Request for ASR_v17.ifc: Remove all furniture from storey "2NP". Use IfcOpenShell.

First a look at what the model holds.

```python
import ifcopenshell
import ifcopenshell.util.element

model = ifcopenshell.open("ASR_v17.ifc")
print(model.schema)
storey = next(s for s in model.by_type("IfcBuildingStorey") if s.Name == "2NP")
furniture = [e for e in ifcopenshell.util.element.get_decomposition(storey) if e.is_a("IfcFurnishingElement")]
seen = {}
for e in furniture:
    element_type = ifcopenshell.util.element.get_type(e)
    name = element_type.Name if element_type not in (None, e) else None
    seen[name] = seen.get(name, 0) + 1
for name, count in sorted(seen.items(), key=str):
    print(count, "x", name)
```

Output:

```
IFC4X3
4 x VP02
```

```python
import ifcopenshell
import ifcopenshell.api.root
import ifcopenshell.util.element

model = ifcopenshell.open("ASR_v17.ifc")

storey = next(s for s in model.by_type("IfcBuildingStorey") if s.Name == "2NP")
furniture = [e for e in ifcopenshell.util.element.get_decomposition(storey) if e.is_a("IfcFurnishingElement")]

for e in furniture:
    ifcopenshell.api.root.remove_product(model, product=e)
print(len(furniture), "removed")

model.write("ASR_v17_updated.ifc")
```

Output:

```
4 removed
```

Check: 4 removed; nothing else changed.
